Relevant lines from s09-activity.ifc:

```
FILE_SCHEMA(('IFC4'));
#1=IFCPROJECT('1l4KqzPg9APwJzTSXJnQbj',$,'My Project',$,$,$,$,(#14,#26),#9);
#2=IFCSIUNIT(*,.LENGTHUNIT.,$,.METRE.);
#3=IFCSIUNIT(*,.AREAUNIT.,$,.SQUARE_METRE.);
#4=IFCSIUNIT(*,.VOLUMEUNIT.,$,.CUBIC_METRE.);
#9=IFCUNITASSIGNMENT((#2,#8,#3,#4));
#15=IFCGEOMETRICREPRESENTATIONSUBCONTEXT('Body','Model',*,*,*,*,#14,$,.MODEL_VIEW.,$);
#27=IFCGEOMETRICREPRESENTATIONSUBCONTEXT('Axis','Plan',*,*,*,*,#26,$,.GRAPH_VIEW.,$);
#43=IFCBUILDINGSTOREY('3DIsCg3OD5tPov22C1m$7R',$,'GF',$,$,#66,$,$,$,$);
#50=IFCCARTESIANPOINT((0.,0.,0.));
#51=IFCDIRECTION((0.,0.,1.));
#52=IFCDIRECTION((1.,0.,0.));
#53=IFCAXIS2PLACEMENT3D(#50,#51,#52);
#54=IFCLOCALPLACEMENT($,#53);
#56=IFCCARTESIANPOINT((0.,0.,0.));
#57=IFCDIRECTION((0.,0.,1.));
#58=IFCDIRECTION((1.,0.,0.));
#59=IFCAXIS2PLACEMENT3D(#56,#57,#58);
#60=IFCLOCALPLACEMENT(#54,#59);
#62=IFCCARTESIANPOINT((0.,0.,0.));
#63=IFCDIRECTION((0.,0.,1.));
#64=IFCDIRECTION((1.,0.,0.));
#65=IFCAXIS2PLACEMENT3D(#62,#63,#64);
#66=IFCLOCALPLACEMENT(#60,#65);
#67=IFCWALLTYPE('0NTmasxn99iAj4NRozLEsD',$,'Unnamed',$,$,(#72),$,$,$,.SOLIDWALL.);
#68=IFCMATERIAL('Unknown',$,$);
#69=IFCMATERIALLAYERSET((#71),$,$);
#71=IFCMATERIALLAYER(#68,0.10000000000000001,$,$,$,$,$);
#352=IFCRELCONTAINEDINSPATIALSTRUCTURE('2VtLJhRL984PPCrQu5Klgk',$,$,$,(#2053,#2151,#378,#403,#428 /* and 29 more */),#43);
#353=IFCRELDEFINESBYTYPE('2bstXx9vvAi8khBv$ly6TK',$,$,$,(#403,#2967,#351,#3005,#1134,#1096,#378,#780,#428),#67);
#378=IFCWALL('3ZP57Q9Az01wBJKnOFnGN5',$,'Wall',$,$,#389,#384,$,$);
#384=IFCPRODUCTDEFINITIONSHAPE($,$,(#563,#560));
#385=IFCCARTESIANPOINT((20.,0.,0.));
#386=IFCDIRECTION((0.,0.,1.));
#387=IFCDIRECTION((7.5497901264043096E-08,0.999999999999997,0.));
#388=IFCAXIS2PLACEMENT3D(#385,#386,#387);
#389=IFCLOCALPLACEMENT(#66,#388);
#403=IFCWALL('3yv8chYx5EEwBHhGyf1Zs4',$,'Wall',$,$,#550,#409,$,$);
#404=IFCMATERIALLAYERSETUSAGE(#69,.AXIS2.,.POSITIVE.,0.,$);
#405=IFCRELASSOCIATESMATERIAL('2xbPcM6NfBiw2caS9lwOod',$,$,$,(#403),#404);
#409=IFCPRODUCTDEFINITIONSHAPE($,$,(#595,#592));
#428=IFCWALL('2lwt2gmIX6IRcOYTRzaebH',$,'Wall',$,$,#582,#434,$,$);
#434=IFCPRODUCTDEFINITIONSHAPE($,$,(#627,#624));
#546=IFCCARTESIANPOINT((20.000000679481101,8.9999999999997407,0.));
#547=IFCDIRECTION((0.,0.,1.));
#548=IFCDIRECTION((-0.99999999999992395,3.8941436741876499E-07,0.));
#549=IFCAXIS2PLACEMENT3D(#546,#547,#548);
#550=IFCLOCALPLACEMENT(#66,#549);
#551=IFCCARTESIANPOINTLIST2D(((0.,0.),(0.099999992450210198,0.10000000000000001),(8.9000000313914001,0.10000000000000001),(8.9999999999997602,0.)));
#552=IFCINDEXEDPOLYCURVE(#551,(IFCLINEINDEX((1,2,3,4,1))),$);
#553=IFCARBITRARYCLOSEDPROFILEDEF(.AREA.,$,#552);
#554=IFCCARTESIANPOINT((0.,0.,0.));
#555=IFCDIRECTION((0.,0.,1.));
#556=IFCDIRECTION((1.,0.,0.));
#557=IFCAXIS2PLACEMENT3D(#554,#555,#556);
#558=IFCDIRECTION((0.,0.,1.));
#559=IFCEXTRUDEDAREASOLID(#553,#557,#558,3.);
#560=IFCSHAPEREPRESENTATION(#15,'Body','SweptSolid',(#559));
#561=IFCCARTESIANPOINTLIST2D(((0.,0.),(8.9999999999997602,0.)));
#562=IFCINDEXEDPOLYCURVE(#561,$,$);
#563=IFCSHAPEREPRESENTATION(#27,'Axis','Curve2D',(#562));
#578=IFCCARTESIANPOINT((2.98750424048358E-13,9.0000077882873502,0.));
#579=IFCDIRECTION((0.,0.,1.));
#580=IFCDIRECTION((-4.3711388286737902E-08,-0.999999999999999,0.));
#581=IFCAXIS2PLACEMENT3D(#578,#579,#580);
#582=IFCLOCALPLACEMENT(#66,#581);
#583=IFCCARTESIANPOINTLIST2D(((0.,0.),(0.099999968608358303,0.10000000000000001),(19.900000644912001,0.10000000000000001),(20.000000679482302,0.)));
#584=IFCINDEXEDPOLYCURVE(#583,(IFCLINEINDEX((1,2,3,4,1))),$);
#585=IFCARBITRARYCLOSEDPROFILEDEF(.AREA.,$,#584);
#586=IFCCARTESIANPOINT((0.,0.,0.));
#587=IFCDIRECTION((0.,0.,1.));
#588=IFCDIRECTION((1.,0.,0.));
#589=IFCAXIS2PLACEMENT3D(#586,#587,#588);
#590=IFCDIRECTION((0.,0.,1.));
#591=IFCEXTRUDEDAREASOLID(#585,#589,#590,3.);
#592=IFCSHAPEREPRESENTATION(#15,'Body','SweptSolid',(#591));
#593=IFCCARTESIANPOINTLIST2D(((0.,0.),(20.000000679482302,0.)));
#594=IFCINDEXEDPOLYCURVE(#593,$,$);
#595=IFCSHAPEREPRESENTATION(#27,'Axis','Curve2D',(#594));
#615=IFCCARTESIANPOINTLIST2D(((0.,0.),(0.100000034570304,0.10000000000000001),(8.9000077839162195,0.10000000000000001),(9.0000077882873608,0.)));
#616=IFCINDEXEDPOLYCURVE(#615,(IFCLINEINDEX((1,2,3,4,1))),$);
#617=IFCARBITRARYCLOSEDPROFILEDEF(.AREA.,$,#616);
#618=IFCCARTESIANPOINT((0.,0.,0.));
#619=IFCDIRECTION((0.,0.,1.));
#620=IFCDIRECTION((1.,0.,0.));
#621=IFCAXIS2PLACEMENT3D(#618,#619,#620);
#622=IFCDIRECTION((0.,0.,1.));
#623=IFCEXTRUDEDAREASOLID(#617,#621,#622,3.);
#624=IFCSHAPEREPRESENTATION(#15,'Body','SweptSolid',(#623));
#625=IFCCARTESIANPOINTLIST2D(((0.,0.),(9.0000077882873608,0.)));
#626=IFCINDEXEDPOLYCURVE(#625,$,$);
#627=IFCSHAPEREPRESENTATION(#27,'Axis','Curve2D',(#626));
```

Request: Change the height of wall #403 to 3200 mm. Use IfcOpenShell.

```python
import ifcopenshell
import ifcopenshell.geom
import ifcopenshell.util.representation
import ifcopenshell.util.shape

model = ifcopenshell.open("s09-activity.ifc")
settings = ifcopenshell.geom.settings()


def volume(element):
    """Net volume in cubic metres, openings subtracted."""
    shape = ifcopenshell.geom.create_shape(settings, element)
    return ifcopenshell.util.shape.get_volume(shape.geometry)


wall = model.by_id(403)
before = volume(wall)

body = ifcopenshell.util.representation.get_representation(wall, "Model", "Body")
solid = body.Items[0]
old_height = solid.Depth
solid.Depth = 3.2
after = volume(wall)

print(f"height {old_height:g} -> {solid.Depth:g}, volume {before:.3f} -> {after:.3f} m3")

model.write("s09-activity-out.ifc")
```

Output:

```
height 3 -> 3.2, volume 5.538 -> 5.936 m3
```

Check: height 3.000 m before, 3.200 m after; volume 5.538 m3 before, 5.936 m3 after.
